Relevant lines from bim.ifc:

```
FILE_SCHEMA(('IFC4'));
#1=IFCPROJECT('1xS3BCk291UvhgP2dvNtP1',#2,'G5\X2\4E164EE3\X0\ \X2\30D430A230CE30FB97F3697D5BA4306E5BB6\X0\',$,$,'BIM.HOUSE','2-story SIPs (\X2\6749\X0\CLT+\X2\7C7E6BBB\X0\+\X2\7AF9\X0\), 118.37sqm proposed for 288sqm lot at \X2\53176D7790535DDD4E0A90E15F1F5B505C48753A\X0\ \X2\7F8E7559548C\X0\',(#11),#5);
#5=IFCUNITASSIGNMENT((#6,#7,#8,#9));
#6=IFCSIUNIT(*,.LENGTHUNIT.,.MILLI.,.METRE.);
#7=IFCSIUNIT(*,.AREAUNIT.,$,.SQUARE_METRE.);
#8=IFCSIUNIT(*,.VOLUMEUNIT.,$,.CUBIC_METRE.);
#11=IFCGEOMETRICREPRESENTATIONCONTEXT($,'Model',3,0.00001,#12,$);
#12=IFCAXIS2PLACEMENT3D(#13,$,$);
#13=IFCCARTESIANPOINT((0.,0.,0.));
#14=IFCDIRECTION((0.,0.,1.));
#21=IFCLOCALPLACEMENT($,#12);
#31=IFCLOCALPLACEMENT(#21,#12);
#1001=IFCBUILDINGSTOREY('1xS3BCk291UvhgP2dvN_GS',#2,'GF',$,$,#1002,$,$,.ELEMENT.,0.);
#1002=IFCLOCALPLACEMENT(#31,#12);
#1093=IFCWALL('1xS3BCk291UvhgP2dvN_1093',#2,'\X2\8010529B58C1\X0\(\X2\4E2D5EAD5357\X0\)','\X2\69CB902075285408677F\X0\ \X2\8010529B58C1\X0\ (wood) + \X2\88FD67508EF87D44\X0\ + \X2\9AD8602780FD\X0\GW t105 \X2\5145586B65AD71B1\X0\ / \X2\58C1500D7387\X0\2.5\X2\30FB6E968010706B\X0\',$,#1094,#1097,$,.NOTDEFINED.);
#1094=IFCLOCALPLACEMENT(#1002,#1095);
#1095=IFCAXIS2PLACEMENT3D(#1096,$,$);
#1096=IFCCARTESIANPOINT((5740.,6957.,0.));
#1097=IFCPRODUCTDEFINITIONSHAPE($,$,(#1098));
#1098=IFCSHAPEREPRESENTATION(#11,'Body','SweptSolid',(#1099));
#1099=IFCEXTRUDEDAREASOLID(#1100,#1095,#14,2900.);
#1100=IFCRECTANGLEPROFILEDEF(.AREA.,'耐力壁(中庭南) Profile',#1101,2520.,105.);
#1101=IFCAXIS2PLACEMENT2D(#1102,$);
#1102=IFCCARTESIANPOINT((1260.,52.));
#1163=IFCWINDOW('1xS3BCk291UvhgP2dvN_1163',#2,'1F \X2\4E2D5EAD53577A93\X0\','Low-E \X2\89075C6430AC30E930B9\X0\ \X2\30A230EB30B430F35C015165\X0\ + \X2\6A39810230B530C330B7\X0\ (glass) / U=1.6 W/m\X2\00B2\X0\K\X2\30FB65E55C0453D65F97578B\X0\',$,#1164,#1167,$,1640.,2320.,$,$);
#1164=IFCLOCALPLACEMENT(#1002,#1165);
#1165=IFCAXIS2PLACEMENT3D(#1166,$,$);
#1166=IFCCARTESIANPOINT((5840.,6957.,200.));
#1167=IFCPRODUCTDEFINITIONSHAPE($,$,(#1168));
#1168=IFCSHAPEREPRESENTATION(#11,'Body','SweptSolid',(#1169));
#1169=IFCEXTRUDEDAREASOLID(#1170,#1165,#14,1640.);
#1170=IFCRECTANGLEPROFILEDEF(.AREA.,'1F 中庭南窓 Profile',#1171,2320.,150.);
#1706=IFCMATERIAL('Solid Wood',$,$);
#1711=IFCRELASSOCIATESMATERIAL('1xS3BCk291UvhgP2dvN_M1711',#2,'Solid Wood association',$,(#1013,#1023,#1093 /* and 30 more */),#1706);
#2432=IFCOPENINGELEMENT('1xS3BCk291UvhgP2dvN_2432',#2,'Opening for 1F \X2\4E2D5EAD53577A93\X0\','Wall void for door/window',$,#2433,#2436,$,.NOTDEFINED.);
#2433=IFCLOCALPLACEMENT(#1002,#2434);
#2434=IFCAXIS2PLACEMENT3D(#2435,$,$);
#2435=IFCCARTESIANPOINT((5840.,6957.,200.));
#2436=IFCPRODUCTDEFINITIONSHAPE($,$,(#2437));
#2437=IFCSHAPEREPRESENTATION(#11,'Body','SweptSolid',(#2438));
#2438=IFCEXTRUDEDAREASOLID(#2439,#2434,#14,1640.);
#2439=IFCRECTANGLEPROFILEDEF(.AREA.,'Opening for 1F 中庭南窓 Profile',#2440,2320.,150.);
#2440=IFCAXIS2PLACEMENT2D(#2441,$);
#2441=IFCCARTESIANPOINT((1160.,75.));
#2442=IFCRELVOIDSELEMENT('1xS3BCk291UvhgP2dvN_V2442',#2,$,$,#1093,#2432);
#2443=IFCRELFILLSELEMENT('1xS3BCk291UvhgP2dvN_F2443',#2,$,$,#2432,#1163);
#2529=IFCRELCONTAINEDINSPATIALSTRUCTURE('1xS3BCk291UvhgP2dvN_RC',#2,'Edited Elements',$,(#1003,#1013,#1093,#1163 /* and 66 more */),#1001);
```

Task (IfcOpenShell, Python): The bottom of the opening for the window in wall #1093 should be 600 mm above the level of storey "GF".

```python
import numpy as np
import ifcopenshell
import ifcopenshell.api.geometry
import ifcopenshell.geom
import ifcopenshell.util.element
import ifcopenshell.util.placement
import ifcopenshell.util.shape
import ifcopenshell.util.unit

model = ifcopenshell.open("bim.ifc")
unit_scale = ifcopenshell.util.unit.calculate_unit_scale(model)

window = model.by_guid("1xS3BCk291UvhgP2dvN_1163")
opening = window.FillsVoids[0].RelatingOpeningElement
storey = ifcopenshell.util.element.get_container(window, ifc_class="IfcBuildingStorey")
level = ifcopenshell.util.placement.get_local_placement(storey.ObjectPlacement)[2, 3]

# The opening's origin need not be at the sill, so measure its lowest point.
shape = ifcopenshell.geom.create_shape(ifcopenshell.geom.settings(), opening)
bottom = ifcopenshell.util.shape.get_shape_bottom_elevation(shape, shape.geometry) / unit_scale
dz = level + 0.6 / unit_scale - bottom

shift = np.array([0.0, 0.0, dz])
# The window is not placed relative to its opening, so move both.
for product in (opening, window):
    matrix = ifcopenshell.util.placement.get_local_placement(product.ObjectPlacement)
    matrix[:3, 3] += shift
    ifcopenshell.api.geometry.edit_object_placement(model, product=product, matrix=matrix, is_si=False)

print(f"moved by {dz * unit_scale:+.3f} m")

model.write("bim_rev.ifc")
```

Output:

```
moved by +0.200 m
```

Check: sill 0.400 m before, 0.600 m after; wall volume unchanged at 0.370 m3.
